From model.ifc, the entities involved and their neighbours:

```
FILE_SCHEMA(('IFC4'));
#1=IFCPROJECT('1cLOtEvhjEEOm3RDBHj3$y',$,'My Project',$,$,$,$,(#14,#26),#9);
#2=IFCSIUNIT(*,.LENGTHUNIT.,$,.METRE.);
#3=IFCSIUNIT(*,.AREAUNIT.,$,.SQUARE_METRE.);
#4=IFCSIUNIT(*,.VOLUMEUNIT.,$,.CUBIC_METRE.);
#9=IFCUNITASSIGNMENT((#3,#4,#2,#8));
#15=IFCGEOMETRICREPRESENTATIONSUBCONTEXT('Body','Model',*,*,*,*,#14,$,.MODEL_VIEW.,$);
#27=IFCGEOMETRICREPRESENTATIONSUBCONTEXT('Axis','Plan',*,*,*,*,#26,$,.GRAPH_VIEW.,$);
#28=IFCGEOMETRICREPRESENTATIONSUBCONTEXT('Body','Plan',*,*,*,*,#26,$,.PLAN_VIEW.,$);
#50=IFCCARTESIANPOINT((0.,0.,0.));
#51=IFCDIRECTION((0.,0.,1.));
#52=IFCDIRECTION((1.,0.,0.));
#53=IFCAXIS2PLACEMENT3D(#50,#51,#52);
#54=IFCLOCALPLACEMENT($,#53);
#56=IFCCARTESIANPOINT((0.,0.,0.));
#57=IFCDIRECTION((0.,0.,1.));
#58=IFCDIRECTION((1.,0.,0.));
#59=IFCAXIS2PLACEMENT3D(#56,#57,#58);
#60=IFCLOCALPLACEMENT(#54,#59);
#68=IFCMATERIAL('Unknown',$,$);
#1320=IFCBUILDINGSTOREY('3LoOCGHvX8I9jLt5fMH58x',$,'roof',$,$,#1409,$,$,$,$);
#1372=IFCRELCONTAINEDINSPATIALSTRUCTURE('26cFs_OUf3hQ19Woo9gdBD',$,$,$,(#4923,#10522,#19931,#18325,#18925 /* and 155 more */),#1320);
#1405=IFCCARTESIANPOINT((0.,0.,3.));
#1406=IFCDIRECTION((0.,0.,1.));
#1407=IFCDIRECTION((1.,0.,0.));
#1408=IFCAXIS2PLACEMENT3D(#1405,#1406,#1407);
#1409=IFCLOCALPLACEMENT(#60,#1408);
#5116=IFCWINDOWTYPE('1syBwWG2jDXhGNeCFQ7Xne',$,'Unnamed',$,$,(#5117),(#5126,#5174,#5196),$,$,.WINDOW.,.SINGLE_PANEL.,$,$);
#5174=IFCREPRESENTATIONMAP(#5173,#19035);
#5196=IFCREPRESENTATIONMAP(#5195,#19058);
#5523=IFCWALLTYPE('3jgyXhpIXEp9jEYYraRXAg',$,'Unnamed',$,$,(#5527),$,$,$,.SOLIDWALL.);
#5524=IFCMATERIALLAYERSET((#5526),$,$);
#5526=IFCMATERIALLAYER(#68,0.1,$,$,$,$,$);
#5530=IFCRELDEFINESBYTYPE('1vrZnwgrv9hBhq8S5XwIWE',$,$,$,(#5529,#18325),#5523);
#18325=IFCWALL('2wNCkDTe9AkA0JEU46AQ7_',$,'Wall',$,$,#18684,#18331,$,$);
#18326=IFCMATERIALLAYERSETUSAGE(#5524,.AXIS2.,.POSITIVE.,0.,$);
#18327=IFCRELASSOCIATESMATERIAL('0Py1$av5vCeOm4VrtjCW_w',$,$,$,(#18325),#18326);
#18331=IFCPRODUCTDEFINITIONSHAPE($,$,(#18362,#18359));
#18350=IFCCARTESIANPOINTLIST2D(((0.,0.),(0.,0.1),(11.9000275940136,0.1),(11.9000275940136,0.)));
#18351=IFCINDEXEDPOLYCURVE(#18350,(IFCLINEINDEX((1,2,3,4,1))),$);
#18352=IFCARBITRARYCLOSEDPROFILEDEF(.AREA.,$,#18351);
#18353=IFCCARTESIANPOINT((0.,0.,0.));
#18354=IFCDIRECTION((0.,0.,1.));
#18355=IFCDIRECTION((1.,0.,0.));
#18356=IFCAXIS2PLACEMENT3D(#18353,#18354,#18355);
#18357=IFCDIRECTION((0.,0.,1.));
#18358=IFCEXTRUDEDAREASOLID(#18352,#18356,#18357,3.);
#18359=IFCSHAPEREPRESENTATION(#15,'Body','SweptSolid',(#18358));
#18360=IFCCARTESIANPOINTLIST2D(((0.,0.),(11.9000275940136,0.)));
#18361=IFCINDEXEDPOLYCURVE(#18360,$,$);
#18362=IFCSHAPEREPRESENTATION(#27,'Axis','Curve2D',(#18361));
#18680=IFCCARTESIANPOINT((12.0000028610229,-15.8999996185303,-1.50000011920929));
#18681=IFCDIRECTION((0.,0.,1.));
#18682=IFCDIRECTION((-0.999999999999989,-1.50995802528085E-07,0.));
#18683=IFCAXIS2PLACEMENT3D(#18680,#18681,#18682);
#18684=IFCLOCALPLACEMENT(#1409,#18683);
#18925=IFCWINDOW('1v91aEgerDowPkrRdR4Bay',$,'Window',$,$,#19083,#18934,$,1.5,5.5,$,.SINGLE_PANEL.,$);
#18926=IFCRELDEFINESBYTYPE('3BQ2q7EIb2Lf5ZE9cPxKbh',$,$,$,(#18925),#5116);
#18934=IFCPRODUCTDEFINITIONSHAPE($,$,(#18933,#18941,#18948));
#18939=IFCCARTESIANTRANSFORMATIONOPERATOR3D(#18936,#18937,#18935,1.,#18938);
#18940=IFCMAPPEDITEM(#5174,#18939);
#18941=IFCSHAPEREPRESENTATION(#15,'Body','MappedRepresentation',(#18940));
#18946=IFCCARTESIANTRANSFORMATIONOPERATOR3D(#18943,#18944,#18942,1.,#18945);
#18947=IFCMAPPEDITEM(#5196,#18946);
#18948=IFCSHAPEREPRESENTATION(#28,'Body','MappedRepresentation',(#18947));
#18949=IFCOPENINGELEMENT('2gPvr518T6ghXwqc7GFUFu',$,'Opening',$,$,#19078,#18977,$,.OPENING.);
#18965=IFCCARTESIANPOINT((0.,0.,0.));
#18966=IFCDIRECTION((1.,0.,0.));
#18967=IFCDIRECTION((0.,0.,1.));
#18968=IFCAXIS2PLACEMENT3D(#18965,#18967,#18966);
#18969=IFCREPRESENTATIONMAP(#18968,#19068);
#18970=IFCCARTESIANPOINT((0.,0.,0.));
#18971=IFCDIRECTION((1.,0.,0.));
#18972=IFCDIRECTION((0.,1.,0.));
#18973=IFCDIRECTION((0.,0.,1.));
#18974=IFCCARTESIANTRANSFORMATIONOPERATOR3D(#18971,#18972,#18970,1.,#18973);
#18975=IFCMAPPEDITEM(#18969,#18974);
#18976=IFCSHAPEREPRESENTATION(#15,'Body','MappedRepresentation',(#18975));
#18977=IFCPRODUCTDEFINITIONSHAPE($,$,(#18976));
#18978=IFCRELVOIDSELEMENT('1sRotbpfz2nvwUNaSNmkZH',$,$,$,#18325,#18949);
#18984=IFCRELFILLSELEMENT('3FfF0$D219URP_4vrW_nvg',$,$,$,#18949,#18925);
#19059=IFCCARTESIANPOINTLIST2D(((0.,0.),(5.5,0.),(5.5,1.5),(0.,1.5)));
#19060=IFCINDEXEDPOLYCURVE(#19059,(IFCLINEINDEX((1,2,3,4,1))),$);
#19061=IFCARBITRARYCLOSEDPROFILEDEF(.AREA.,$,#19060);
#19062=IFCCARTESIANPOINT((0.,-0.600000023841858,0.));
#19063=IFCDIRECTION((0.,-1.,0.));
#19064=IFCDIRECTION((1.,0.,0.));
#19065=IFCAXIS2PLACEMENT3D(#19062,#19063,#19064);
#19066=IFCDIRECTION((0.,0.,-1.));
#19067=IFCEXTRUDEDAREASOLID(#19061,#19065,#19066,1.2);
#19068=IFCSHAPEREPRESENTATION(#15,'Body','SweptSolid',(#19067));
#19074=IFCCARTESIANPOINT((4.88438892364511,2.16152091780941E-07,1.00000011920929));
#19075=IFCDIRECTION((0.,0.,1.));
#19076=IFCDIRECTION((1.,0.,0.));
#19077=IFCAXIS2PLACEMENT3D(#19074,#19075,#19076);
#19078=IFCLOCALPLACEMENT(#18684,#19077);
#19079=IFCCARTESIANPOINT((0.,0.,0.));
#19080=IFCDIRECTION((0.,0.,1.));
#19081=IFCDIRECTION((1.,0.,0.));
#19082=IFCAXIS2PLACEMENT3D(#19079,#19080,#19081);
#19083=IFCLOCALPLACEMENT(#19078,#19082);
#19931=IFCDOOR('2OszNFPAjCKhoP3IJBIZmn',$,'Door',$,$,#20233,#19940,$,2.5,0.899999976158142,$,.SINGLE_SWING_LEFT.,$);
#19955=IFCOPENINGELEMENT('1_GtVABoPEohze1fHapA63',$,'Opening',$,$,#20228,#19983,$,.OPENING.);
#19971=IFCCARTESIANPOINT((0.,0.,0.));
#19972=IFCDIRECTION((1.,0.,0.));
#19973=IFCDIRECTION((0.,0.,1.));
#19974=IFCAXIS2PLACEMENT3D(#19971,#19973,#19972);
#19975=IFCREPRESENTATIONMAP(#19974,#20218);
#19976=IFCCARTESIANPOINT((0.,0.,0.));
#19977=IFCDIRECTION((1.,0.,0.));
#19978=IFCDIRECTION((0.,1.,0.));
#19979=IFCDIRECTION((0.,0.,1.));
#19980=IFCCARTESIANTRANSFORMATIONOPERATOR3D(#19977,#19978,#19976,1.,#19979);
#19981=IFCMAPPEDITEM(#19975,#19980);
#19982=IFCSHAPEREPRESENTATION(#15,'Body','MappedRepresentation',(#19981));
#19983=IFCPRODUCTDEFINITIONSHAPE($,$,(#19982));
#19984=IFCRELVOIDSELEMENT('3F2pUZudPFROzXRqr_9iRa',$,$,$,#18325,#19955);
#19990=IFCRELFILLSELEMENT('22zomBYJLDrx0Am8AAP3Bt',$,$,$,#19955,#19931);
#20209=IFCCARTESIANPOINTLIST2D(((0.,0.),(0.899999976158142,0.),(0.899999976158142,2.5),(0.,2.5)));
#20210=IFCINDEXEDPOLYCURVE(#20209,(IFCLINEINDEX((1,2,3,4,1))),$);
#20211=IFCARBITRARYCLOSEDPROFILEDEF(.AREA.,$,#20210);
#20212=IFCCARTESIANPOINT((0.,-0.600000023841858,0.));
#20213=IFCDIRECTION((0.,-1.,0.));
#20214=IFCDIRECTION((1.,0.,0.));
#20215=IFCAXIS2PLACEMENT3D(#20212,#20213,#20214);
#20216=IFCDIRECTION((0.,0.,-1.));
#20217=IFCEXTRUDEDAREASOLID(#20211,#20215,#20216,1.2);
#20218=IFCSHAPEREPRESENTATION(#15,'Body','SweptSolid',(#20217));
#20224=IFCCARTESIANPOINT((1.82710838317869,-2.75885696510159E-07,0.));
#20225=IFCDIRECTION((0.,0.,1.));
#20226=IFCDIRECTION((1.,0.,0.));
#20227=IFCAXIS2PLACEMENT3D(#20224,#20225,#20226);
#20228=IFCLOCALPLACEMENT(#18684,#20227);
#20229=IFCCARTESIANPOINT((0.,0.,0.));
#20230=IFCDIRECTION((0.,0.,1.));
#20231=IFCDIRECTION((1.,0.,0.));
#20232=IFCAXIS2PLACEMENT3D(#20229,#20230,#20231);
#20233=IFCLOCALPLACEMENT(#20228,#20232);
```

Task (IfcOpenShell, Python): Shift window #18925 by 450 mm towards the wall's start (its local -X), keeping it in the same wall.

```python
import ifcopenshell
import ifcopenshell.api.geometry
import ifcopenshell.util.placement
import ifcopenshell.util.unit

model = ifcopenshell.open("model.ifc")
unit_scale = ifcopenshell.util.unit.calculate_unit_scale(model)

window = model.by_guid("1v91aEgerDowPkrRdR4Bay")
opening = window.FillsVoids[0].RelatingOpeningElement
wall = opening.VoidsElements[0].RelatingBuildingElement

wall_matrix = ifcopenshell.util.placement.get_local_placement(wall.ObjectPlacement)
shift = wall_matrix[:3, 0] * -0.45 / unit_scale
before = ifcopenshell.util.placement.get_local_placement(window.ObjectPlacement)[:3, 3].copy()

# The window is placed relative to its opening, so it follows when the opening moves.
matrix = ifcopenshell.util.placement.get_local_placement(opening.ObjectPlacement)
matrix[:3, 3] += shift
ifcopenshell.api.geometry.edit_object_placement(
    model, product=opening, matrix=matrix, is_si=False, should_transform_children=True
)

after = ifcopenshell.util.placement.get_local_placement(window.ObjectPlacement)[:3, 3]
print("window moved by", (after - before).round(3) + 0.0)

model.write("model_edited.ifc")
```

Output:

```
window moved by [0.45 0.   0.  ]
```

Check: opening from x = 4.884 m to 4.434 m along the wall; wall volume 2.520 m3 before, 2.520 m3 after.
